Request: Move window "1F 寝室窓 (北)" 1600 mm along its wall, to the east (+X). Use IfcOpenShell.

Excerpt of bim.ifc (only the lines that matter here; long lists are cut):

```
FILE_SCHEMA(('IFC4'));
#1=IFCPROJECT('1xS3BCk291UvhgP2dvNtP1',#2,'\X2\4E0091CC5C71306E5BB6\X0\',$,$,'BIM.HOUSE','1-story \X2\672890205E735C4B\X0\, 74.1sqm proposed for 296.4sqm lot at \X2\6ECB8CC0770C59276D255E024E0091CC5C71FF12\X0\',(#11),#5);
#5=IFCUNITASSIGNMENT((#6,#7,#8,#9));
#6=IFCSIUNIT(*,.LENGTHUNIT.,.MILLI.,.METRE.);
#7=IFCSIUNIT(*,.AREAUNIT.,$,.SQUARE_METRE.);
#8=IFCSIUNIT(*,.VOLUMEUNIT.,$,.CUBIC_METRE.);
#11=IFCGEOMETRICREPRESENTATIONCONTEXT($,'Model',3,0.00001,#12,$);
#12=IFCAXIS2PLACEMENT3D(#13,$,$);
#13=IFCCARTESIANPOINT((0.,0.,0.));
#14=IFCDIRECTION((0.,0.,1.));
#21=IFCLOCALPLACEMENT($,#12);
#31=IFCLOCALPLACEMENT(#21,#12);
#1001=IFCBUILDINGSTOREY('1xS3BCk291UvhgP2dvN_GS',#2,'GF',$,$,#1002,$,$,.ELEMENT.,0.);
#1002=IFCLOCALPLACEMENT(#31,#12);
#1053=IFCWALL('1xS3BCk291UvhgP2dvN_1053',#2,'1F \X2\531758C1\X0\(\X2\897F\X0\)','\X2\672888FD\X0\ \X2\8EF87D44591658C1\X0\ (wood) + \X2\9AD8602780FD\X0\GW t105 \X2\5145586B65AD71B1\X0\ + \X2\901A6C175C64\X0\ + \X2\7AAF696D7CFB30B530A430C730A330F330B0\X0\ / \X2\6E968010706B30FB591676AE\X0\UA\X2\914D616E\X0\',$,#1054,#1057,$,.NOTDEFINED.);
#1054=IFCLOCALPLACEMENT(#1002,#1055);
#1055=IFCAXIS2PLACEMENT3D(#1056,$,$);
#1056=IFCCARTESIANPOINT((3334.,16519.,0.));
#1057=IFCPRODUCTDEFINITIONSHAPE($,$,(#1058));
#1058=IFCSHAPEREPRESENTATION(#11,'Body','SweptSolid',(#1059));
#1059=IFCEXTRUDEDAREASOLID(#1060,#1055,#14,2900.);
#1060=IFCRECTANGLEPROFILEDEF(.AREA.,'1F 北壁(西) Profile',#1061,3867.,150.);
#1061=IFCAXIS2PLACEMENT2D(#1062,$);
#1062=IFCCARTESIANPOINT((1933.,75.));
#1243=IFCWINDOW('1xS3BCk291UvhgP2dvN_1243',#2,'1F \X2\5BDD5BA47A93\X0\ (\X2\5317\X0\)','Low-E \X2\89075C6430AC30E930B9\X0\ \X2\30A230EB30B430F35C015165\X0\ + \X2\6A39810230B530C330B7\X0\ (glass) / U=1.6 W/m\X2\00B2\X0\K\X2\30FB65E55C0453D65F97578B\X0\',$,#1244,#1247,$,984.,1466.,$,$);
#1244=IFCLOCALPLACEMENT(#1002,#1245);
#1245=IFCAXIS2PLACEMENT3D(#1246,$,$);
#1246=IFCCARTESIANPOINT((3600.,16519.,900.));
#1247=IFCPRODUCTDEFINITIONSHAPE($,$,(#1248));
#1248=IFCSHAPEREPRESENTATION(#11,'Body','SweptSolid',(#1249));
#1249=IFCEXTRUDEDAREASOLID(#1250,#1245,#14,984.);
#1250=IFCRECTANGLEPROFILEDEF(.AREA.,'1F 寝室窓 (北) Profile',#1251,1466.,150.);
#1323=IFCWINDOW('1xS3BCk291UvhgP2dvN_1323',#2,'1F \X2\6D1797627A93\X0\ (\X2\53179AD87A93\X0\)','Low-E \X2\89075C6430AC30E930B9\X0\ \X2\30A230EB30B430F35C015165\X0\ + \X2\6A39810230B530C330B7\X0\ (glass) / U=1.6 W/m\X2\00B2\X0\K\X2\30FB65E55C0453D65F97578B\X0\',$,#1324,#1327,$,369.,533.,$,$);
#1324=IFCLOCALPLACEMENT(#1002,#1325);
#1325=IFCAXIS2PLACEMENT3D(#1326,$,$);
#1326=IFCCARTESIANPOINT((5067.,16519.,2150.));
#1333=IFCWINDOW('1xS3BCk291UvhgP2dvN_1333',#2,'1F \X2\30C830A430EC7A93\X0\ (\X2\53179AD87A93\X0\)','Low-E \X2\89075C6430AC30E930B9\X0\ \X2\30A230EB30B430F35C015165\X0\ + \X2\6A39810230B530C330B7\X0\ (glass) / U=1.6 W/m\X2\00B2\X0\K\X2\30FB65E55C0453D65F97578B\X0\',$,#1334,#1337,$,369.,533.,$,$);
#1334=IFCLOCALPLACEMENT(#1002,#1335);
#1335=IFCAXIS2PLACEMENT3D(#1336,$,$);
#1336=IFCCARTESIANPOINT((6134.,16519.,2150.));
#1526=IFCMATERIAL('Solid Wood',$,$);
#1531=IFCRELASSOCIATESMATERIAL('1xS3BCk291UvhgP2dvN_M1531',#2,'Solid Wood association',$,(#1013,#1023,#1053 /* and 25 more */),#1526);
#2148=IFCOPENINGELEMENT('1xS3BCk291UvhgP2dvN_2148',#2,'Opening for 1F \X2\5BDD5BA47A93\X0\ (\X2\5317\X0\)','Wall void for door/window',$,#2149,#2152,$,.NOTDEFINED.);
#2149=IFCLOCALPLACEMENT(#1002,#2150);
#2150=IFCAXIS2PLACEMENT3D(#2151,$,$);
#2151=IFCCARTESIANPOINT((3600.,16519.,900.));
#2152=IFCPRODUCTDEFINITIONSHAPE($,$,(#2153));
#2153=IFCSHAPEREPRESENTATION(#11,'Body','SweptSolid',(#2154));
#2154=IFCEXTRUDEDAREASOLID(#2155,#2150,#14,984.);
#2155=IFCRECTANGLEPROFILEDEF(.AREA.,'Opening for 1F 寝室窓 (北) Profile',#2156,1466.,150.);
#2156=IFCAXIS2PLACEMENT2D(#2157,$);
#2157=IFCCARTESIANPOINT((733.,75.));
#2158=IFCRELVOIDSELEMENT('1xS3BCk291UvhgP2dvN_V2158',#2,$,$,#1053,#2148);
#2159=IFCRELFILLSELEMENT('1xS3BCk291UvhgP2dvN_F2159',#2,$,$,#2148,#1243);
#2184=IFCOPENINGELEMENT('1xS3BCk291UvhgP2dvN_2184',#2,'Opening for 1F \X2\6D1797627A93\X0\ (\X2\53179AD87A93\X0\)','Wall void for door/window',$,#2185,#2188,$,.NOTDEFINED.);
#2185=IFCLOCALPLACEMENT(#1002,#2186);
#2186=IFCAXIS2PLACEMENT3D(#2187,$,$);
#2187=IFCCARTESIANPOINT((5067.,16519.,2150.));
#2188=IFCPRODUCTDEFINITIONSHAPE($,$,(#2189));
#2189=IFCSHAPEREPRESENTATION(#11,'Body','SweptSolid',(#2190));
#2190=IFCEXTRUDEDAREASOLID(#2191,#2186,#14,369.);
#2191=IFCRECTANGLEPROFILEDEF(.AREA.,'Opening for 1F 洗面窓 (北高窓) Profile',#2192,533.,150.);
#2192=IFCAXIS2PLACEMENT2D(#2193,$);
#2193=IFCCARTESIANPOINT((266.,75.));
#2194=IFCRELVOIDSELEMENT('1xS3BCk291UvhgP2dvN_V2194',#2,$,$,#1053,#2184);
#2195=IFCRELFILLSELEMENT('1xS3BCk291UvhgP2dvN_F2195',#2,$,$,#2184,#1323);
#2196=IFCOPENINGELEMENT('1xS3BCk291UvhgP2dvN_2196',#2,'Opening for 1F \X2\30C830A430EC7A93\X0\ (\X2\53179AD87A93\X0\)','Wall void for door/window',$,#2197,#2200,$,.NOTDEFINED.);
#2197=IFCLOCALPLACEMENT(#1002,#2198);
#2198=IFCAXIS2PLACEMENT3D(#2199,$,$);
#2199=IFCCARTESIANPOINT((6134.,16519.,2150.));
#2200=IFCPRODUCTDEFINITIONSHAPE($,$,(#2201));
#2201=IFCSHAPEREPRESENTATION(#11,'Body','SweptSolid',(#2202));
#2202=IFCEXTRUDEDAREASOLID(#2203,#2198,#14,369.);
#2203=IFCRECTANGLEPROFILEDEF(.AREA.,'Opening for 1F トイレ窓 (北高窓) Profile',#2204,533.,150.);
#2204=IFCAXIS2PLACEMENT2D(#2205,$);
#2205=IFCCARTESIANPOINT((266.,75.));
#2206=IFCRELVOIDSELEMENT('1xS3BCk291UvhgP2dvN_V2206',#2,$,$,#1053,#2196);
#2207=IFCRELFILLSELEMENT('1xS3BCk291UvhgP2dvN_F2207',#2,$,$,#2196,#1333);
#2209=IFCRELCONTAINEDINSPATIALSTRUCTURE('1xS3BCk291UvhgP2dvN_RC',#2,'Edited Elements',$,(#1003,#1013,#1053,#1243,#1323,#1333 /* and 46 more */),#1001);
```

```python
import ifcopenshell
import ifcopenshell.api.geometry
import ifcopenshell.util.placement

model = ifcopenshell.open("bim.ifc")

window = model.by_guid("1xS3BCk291UvhgP2dvN_1243")
opening = window.FillsVoids[0].RelatingOpeningElement
wall = opening.VoidsElements[0].RelatingBuildingElement

wall_matrix = ifcopenshell.util.placement.get_local_placement(wall.ObjectPlacement)
shift = wall_matrix[:3, 0] * 1600.0
before = ifcopenshell.util.placement.get_local_placement(window.ObjectPlacement)[:3, 3].copy()

# The window is not placed relative to its opening, so move both.
for product in (opening, window):
    matrix = ifcopenshell.util.placement.get_local_placement(product.ObjectPlacement)
    matrix[:3, 3] += shift
    ifcopenshell.api.geometry.edit_object_placement(model, product=product, matrix=matrix, is_si=False)

after = ifcopenshell.util.placement.get_local_placement(window.ObjectPlacement)[:3, 3]
print("window moved by", (after - before).round(3) + 0.0)

model.write("bim_v2.ifc")
```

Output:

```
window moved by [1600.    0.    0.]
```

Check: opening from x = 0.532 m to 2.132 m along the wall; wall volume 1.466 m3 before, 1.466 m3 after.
